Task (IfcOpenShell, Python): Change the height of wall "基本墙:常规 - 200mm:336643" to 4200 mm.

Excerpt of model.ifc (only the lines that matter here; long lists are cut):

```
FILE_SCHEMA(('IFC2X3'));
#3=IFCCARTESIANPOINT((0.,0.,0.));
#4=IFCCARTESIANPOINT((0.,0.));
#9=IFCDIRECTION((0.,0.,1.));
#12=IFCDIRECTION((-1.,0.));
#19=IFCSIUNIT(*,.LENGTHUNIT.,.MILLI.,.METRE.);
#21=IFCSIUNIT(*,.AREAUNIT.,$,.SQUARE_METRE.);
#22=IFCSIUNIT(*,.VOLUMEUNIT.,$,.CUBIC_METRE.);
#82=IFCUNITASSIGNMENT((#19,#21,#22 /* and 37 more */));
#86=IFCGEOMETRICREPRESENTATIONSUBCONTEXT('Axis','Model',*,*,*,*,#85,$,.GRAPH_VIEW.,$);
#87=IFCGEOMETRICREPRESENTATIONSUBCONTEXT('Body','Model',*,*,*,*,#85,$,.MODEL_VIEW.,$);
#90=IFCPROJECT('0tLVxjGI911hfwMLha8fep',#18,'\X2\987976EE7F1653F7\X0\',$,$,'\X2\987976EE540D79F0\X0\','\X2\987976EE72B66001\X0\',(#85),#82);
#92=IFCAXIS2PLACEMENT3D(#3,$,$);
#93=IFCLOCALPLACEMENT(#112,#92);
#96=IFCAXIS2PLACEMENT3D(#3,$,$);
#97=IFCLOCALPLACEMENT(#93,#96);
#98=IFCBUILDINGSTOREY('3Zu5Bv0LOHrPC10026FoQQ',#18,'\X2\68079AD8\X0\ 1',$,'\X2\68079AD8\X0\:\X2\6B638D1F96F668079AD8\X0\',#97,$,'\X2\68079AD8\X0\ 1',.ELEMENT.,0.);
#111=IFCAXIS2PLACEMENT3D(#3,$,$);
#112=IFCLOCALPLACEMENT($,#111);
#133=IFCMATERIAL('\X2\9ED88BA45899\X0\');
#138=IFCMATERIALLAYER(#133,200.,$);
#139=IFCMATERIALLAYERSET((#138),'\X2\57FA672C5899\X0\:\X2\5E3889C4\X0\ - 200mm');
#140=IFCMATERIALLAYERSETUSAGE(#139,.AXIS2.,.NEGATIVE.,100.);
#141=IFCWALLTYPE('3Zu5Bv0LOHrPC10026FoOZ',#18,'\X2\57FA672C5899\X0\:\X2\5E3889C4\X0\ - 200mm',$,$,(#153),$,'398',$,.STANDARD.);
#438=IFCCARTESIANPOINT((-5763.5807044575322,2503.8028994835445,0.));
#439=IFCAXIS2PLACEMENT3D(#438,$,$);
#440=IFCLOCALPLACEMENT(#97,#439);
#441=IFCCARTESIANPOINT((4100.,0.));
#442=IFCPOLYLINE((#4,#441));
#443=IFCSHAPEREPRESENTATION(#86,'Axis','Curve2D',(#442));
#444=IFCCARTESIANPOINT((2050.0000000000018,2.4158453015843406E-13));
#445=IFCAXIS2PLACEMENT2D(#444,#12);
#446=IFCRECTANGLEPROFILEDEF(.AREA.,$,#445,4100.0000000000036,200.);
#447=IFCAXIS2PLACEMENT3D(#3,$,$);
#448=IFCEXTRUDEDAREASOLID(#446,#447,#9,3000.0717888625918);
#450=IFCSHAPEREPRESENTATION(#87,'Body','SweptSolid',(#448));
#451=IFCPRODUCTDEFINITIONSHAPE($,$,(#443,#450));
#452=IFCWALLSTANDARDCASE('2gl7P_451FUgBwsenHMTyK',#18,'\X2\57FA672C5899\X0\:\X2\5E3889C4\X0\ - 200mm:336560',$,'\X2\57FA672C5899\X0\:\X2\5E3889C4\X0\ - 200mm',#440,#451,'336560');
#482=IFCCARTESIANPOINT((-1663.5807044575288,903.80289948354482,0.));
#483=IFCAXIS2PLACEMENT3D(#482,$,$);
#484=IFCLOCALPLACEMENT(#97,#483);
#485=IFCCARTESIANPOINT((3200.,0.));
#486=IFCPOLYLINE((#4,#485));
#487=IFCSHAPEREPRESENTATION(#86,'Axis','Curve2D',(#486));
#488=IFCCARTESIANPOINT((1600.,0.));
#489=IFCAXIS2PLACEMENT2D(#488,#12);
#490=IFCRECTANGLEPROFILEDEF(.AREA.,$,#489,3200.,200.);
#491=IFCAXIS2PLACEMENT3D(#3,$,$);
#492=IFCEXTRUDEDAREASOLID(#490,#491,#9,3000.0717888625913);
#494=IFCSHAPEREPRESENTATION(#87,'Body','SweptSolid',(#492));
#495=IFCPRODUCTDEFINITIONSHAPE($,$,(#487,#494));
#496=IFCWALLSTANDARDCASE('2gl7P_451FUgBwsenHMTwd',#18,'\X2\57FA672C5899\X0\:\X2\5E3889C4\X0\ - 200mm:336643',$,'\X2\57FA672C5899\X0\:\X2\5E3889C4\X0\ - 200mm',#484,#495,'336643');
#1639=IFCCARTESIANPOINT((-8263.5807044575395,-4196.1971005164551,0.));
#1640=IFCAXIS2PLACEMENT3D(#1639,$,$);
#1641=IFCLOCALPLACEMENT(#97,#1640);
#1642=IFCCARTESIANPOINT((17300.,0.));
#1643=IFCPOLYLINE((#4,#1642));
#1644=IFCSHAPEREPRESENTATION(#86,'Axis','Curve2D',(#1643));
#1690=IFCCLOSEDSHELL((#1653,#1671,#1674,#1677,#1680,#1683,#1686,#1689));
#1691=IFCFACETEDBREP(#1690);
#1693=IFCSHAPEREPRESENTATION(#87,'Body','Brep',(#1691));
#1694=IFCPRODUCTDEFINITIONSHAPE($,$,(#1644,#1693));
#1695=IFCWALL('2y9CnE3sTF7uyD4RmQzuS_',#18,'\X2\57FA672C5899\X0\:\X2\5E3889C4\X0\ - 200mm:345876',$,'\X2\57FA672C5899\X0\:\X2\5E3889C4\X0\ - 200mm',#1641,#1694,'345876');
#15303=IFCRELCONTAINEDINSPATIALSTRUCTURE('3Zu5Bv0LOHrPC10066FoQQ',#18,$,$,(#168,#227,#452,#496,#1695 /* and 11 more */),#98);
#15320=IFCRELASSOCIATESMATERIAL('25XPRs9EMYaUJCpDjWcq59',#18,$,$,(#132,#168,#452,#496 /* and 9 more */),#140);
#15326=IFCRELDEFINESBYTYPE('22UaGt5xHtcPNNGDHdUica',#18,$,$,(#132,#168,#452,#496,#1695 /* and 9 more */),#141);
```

```python
import ifcopenshell
import ifcopenshell.geom
import ifcopenshell.util.representation
import ifcopenshell.util.shape

model = ifcopenshell.open("model.ifc")
settings = ifcopenshell.geom.settings()


def volume(element):
    """Net volume in cubic metres, openings subtracted."""
    shape = ifcopenshell.geom.create_shape(settings, element)
    return ifcopenshell.util.shape.get_volume(shape.geometry)


wall = model.by_guid("2gl7P_451FUgBwsenHMTwd")
before = volume(wall)

body = ifcopenshell.util.representation.get_representation(wall, "Model", "Body")
solid = body.Items[0]
old_height = solid.Depth
solid.Depth = 4200.0
after = volume(wall)

print(f"height {old_height:g} -> {solid.Depth:g}, volume {before:.3f} -> {after:.3f} m3")

model.write("model_updated.ifc")
```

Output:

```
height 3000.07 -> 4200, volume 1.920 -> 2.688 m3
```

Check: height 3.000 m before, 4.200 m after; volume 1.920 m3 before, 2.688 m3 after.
